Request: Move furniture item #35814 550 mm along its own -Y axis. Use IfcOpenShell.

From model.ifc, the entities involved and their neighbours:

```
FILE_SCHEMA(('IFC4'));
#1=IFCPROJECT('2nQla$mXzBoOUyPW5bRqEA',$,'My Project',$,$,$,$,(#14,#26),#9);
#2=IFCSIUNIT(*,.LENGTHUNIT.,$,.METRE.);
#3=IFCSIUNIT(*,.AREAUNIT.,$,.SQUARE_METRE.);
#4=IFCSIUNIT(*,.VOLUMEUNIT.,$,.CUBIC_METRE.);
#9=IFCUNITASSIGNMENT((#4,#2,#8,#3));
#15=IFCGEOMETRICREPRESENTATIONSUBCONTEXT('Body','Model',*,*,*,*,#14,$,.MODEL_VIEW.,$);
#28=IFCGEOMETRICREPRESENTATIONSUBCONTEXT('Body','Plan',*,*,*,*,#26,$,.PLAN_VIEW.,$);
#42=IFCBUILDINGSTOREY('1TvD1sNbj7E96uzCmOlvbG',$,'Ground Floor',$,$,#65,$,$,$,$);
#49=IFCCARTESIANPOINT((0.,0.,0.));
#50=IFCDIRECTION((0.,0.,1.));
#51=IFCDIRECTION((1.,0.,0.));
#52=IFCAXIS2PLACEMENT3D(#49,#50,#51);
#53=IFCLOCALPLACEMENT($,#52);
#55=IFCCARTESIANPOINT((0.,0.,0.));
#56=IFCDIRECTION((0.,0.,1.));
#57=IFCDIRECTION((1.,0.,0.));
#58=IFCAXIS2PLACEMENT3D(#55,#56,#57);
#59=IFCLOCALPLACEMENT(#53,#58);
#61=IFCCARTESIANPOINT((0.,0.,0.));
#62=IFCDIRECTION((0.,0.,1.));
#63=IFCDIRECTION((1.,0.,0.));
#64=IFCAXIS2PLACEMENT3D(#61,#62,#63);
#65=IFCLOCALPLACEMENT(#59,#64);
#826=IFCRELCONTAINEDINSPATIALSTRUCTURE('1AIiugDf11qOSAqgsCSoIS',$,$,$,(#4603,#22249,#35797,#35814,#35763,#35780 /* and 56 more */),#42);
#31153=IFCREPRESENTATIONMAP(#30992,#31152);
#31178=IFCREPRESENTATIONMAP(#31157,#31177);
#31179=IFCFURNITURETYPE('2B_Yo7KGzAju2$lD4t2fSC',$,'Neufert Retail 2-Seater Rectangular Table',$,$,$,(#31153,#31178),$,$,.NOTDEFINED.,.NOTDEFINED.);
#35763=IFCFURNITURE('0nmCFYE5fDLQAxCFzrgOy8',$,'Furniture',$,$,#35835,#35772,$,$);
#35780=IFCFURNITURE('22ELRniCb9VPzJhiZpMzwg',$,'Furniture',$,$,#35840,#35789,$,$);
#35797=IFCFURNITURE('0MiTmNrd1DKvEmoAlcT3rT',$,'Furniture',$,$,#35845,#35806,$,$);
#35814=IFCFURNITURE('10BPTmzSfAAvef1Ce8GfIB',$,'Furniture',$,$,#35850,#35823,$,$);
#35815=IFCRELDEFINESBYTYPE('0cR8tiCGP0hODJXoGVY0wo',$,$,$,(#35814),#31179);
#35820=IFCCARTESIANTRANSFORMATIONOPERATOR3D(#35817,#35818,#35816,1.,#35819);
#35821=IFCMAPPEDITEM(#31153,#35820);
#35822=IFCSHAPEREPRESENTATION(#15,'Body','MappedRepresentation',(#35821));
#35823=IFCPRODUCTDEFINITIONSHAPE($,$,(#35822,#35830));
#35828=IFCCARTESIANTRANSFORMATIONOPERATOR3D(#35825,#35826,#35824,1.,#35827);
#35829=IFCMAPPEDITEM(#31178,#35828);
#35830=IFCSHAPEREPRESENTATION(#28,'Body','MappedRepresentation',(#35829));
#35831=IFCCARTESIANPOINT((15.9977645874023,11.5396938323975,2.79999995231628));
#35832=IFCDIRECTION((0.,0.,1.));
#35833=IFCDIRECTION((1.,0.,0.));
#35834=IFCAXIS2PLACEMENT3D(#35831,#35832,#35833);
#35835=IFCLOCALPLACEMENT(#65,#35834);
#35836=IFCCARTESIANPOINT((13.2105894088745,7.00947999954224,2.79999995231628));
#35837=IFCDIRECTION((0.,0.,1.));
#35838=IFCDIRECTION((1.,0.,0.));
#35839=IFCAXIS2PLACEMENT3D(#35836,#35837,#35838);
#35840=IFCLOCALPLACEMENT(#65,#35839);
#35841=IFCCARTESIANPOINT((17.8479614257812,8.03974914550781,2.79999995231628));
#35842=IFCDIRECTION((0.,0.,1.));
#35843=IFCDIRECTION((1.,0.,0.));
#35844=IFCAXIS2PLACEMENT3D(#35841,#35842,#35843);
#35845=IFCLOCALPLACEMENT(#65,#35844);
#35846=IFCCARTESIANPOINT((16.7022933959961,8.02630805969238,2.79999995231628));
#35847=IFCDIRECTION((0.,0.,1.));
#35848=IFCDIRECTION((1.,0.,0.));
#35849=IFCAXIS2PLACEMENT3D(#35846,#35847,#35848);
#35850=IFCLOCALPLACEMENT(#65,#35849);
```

```python
import ifcopenshell
import ifcopenshell.api.geometry
import ifcopenshell.util.placement
import ifcopenshell.util.unit

model = ifcopenshell.open("model.ifc")
unit_scale = ifcopenshell.util.unit.calculate_unit_scale(model)

item = model.by_id(35814)
matrix = ifcopenshell.util.placement.get_local_placement(item.ObjectPlacement)
matrix[:3, 3] -= matrix[:3, 1] * 0.55 / unit_scale
ifcopenshell.api.geometry.edit_object_placement(model, product=item, matrix=matrix, is_si=False)

print(ifcopenshell.util.placement.get_local_placement(item.ObjectPlacement).round(3) + 0.0)

model.write("model_rev.ifc")
```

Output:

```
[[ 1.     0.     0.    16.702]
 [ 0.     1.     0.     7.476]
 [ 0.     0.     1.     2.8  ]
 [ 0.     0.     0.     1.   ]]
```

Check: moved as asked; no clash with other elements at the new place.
